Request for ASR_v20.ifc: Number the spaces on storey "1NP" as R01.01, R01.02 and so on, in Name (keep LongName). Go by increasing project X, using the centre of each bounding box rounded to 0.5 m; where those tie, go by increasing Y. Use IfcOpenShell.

First a look at what the model holds.

```python
import ifcopenshell
import ifcopenshell.util.element
import ifcopenshell.util.placement

model = ifcopenshell.open("ASR_v20.ifc")
print(model.schema)
storey = next(s for s in model.by_type("IfcBuildingStorey") if s.Name == "1NP")
spaces = [e for e in ifcopenshell.util.element.get_decomposition(storey) if e.is_a("IfcSpace")]
for e in sorted(spaces, key=lambda e: e.id()):
    origin = ifcopenshell.util.placement.get_local_placement(e.ObjectPlacement)[:3, 3]
    print(e.id(), e.Name, e.LongName, origin.round(2) + 0.0, sep=" | ")
```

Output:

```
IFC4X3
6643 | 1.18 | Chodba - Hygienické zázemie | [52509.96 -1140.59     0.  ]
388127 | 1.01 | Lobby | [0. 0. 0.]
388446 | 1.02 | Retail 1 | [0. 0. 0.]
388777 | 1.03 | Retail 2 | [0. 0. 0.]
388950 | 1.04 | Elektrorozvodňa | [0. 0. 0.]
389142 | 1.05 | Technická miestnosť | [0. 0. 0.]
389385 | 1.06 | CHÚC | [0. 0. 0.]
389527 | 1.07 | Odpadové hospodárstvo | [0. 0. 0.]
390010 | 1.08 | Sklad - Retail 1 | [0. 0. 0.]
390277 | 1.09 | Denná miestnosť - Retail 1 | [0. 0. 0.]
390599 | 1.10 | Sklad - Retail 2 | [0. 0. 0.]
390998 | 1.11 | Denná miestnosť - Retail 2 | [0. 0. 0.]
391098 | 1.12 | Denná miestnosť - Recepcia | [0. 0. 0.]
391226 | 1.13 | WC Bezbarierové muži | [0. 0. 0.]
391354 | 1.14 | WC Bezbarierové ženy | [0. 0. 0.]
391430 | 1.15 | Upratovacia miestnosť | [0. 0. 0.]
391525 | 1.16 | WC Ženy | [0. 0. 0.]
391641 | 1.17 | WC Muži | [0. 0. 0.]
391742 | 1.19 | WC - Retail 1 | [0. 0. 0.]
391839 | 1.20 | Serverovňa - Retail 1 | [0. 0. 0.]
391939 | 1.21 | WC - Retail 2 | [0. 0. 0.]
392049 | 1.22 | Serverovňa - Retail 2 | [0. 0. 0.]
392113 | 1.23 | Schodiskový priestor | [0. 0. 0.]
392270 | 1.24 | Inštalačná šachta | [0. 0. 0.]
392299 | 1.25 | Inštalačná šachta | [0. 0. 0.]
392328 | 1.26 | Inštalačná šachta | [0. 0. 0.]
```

```python
import ifcopenshell
import ifcopenshell.geom
import ifcopenshell.util.element
import ifcopenshell.util.shape

model = ifcopenshell.open("ASR_v20.ifc")
settings = ifcopenshell.geom.settings()
settings.set("use-world-coords", True)


def centre(element):
    shape = ifcopenshell.geom.create_shape(settings, element)
    return ifcopenshell.util.shape.get_bbox_centroid(shape.geometry)


storey = next(s for s in model.by_type("IfcBuildingStorey") if s.Name == "1NP")
spaces = [e for e in ifcopenshell.util.element.get_decomposition(storey) if e.is_a("IfcSpace")]

# Insertion points can sit at a corner or the storey origin, so sort by the geometry (in metres).
centres = {e: centre(e) for e in spaces}
spaces.sort(key=lambda e: (round(centres[e][0] / 0.5), centres[e][1]))

for i, e in enumerate(spaces, start=1):
    number = f"R01.{i:02d}"
    e.Name = number
    print(e.id(), number)

model.write("ASR_v20_edited.ifc")
```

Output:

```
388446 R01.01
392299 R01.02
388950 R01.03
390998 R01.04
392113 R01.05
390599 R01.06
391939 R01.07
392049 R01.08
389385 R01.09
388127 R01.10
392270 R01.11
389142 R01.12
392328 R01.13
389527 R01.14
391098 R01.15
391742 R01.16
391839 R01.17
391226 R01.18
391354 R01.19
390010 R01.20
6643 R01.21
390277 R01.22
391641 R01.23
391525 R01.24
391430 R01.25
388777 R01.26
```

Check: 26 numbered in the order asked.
